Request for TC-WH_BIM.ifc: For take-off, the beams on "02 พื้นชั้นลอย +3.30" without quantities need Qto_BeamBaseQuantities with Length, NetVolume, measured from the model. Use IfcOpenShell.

First a look at what the model holds.

```python
import ifcopenshell
import ifcopenshell.util.element
import ifcopenshell.util.unit

model = ifcopenshell.open("TC-WH_BIM.ifc")
print(model.schema)
for unit_type in ("LENGTHUNIT", "AREAUNIT", "VOLUMEUNIT"):
    print(unit_type, ifcopenshell.util.unit.calculate_unit_scale(model, unit_type))
storey = next(s for s in model.by_type("IfcBuildingStorey") if s.Name == "02 พื้นชั้นลอย +3.30")
beams = [e for e in ifcopenshell.util.element.get_decomposition(storey) if e.is_a("IfcBeam")]
for e in sorted(beams, key=lambda e: e.id()):
    print(e.id(), e.is_a(), e.Name, list(ifcopenshell.util.element.get_psets(e, qtos_only=True)), sep=" | ")
```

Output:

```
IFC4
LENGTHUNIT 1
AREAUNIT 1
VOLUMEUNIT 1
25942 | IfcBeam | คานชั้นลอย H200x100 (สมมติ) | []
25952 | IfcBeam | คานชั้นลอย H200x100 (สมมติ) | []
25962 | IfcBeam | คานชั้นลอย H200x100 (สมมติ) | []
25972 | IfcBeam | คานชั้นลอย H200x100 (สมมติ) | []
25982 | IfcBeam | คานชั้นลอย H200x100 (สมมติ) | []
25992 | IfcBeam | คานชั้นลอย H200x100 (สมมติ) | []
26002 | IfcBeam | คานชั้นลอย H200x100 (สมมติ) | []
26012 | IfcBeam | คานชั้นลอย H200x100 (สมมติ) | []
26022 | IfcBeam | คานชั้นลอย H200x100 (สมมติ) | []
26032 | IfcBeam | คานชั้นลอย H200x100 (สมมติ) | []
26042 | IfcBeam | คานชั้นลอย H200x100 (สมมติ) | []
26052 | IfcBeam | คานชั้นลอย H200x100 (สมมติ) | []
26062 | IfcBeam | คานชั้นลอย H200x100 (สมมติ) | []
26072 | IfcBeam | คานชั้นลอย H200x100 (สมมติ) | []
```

```python
import ifcopenshell
import ifcopenshell.api.pset
import ifcopenshell.geom
import ifcopenshell.util.element
import ifcopenshell.util.shape
import ifcopenshell.util.unit

model = ifcopenshell.open("TC-WH_BIM.ifc")
unit_scale = ifcopenshell.util.unit.calculate_unit_scale(model)
volume_scale = ifcopenshell.util.unit.calculate_unit_scale(model, "VOLUMEUNIT")
settings = ifcopenshell.geom.settings()

storey = next(s for s in model.by_type("IfcBuildingStorey") if s.Name == "02 พื้นชั้นลอย +3.30")
beams = [e for e in ifcopenshell.util.element.get_decomposition(storey) if e.is_a("IfcBeam")]

for e in sorted(beams, key=lambda e: e.id()):
    if ifcopenshell.util.element.get_psets(e, qtos_only=True, should_inherit=False):
        continue
    # Geometry comes back in metres, in the element's own axes.
    shape = ifcopenshell.geom.create_shape(settings, e)
    values = {
        "Length": ifcopenshell.util.shape.get_max_xyz(shape.geometry) / unit_scale,
        "NetVolume": ifcopenshell.util.shape.get_volume(shape.geometry) / volume_scale,
    }
    qto = ifcopenshell.api.pset.add_qto(model, product=e, name="Qto_BeamBaseQuantities")
    ifcopenshell.api.pset.edit_qto(model, qto=qto, properties=values)
    print(e.id(), {k: round(v, 3) for k, v in values.items()})

model.write("TC-WH_BIM_rev.ifc")
```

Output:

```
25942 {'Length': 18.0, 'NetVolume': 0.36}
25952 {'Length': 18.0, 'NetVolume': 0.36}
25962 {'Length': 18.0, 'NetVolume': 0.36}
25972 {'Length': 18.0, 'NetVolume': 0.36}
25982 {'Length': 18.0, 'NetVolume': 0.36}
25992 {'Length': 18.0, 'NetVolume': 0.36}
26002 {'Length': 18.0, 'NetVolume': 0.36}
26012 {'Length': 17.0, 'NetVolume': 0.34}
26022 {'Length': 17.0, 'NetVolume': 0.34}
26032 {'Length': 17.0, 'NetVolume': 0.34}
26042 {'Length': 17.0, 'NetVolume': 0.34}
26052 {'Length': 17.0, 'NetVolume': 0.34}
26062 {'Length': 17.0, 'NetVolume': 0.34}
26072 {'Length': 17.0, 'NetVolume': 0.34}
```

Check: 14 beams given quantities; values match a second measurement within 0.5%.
